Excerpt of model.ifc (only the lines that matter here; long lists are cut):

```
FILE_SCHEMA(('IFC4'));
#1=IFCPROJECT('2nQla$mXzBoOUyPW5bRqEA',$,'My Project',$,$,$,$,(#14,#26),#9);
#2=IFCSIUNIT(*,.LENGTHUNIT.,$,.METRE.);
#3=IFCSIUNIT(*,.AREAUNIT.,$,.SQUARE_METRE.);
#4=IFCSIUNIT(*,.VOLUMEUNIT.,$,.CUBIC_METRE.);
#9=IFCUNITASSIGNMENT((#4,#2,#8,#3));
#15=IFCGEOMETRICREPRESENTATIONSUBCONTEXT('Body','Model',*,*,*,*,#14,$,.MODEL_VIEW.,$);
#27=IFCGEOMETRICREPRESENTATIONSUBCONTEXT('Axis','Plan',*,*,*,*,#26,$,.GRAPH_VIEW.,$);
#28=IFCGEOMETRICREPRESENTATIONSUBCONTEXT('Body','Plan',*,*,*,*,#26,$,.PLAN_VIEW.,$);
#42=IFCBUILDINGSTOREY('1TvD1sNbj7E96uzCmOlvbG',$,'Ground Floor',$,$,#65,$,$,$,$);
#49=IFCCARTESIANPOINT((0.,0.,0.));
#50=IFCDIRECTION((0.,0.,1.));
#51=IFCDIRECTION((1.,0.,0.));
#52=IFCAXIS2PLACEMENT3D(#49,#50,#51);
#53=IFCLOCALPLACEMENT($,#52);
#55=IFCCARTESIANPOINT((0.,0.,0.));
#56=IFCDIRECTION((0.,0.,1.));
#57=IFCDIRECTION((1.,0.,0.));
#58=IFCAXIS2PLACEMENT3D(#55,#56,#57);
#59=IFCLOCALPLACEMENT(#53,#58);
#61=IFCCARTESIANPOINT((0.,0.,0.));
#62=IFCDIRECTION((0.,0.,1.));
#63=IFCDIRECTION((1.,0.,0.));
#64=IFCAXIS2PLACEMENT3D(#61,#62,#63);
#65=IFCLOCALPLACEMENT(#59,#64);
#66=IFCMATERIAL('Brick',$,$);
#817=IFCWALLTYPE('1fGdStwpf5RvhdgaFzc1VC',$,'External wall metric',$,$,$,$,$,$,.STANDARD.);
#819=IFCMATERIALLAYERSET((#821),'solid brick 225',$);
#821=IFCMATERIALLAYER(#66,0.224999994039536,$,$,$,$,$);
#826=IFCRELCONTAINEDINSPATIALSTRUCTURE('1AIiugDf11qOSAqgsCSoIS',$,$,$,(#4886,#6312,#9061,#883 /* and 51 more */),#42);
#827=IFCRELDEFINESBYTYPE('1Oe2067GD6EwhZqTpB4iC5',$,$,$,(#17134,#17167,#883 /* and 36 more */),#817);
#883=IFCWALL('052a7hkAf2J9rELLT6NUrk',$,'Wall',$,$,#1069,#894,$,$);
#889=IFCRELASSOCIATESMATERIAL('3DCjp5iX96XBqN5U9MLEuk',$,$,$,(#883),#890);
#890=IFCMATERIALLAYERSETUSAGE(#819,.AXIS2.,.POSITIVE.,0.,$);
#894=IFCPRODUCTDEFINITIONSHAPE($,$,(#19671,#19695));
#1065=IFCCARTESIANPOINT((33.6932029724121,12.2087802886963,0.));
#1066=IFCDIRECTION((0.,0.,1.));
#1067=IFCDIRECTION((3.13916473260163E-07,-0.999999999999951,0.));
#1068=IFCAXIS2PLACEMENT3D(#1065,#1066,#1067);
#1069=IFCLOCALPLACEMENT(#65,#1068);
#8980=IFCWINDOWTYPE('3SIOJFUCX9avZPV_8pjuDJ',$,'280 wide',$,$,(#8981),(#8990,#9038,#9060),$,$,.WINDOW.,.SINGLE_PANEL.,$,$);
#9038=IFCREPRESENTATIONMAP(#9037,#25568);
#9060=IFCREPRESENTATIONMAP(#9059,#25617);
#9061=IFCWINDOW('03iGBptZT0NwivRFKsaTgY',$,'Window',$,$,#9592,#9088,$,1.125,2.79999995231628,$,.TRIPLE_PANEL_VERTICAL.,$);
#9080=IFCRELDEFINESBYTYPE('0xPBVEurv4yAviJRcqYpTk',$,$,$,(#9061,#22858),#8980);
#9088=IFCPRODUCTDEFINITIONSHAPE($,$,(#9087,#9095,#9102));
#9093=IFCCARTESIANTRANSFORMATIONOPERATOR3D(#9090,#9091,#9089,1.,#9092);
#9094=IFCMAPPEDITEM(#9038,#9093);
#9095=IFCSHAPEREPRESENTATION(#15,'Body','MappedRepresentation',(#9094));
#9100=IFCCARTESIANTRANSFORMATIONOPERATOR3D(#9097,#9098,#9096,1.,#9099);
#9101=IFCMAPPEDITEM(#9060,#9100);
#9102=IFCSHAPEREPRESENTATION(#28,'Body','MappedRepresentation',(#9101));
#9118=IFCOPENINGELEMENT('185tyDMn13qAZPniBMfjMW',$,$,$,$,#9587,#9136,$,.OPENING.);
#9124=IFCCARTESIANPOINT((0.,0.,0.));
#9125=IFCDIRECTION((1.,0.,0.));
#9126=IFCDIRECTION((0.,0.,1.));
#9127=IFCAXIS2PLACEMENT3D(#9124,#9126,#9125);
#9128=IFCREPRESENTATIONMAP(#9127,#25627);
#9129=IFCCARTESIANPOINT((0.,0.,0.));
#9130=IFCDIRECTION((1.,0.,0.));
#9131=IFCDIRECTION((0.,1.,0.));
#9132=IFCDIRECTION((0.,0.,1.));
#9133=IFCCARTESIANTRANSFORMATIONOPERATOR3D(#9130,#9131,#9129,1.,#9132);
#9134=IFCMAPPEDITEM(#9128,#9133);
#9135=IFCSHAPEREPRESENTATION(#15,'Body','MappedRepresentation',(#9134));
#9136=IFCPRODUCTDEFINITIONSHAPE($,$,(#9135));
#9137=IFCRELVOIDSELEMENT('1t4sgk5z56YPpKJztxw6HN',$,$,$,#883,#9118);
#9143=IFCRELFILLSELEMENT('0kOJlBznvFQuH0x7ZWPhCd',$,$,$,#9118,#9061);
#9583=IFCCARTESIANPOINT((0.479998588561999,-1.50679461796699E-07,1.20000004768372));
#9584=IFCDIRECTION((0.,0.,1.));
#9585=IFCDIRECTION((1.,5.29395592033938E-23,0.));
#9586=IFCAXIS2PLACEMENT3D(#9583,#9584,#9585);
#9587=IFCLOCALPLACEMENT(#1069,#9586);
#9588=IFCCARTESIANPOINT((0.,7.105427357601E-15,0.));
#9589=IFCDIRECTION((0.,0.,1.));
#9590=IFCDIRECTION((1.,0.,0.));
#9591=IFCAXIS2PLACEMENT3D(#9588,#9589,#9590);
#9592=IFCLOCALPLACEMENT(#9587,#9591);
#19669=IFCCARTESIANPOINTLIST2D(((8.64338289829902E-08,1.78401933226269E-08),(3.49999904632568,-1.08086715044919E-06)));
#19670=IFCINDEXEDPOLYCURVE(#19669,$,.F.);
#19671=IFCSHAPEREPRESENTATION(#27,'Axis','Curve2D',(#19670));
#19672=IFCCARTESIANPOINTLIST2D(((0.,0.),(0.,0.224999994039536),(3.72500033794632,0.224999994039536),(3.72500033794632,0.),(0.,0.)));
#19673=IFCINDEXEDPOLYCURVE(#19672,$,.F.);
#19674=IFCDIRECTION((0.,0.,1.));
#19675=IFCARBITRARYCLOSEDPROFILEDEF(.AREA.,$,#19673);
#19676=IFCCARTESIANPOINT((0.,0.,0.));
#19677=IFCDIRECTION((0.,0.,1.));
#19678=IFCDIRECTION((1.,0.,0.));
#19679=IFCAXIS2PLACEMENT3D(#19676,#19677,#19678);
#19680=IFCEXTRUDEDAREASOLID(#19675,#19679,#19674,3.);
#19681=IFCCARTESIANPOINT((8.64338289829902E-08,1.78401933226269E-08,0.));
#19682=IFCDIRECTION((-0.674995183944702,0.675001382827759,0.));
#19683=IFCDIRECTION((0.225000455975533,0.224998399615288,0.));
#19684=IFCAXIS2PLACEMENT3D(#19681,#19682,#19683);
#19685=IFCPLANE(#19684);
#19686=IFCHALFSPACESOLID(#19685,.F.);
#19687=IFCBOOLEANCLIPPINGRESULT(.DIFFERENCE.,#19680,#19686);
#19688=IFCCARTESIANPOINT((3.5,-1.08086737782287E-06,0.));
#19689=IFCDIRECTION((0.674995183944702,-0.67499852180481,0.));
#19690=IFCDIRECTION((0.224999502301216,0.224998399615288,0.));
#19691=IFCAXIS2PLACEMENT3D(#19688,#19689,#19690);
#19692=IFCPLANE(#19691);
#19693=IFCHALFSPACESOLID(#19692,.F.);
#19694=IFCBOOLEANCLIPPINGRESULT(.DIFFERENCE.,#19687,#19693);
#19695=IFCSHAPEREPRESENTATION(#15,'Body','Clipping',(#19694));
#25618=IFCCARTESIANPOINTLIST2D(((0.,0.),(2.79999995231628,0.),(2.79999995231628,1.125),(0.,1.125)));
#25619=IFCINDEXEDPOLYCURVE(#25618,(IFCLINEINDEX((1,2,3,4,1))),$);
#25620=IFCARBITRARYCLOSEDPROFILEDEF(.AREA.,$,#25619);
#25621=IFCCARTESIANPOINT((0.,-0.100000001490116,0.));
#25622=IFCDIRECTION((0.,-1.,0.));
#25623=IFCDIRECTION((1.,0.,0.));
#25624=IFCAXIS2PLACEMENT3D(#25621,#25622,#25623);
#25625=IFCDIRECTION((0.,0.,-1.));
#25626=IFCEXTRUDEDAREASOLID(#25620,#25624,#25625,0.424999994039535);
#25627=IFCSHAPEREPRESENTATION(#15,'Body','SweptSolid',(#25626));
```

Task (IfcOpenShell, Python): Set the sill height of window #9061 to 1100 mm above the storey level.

```python
import numpy as np
import ifcopenshell
import ifcopenshell.api.geometry
import ifcopenshell.geom
import ifcopenshell.util.element
import ifcopenshell.util.placement
import ifcopenshell.util.shape
import ifcopenshell.util.unit

model = ifcopenshell.open("model.ifc")
unit_scale = ifcopenshell.util.unit.calculate_unit_scale(model)

window = model.by_guid("03iGBptZT0NwivRFKsaTgY")
opening = window.FillsVoids[0].RelatingOpeningElement
storey = ifcopenshell.util.element.get_container(window, ifc_class="IfcBuildingStorey")
level = ifcopenshell.util.placement.get_local_placement(storey.ObjectPlacement)[2, 3]

# The opening's origin need not be at the sill, so measure its lowest point.
shape = ifcopenshell.geom.create_shape(ifcopenshell.geom.settings(), opening)
bottom = ifcopenshell.util.shape.get_shape_bottom_elevation(shape, shape.geometry) / unit_scale
dz = level + 1.1 / unit_scale - bottom

shift = np.array([0.0, 0.0, dz])
# The window is placed relative to its opening, so it follows when the opening moves.
matrix = ifcopenshell.util.placement.get_local_placement(opening.ObjectPlacement)
matrix[:3, 3] += shift
ifcopenshell.api.geometry.edit_object_placement(
    model, product=opening, matrix=matrix, is_si=False, should_transform_children=True
)

print(f"moved by {dz * unit_scale:+.3f} m")

model.write("model-out.ifc")
```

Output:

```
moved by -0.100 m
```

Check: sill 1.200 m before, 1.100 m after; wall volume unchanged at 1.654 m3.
